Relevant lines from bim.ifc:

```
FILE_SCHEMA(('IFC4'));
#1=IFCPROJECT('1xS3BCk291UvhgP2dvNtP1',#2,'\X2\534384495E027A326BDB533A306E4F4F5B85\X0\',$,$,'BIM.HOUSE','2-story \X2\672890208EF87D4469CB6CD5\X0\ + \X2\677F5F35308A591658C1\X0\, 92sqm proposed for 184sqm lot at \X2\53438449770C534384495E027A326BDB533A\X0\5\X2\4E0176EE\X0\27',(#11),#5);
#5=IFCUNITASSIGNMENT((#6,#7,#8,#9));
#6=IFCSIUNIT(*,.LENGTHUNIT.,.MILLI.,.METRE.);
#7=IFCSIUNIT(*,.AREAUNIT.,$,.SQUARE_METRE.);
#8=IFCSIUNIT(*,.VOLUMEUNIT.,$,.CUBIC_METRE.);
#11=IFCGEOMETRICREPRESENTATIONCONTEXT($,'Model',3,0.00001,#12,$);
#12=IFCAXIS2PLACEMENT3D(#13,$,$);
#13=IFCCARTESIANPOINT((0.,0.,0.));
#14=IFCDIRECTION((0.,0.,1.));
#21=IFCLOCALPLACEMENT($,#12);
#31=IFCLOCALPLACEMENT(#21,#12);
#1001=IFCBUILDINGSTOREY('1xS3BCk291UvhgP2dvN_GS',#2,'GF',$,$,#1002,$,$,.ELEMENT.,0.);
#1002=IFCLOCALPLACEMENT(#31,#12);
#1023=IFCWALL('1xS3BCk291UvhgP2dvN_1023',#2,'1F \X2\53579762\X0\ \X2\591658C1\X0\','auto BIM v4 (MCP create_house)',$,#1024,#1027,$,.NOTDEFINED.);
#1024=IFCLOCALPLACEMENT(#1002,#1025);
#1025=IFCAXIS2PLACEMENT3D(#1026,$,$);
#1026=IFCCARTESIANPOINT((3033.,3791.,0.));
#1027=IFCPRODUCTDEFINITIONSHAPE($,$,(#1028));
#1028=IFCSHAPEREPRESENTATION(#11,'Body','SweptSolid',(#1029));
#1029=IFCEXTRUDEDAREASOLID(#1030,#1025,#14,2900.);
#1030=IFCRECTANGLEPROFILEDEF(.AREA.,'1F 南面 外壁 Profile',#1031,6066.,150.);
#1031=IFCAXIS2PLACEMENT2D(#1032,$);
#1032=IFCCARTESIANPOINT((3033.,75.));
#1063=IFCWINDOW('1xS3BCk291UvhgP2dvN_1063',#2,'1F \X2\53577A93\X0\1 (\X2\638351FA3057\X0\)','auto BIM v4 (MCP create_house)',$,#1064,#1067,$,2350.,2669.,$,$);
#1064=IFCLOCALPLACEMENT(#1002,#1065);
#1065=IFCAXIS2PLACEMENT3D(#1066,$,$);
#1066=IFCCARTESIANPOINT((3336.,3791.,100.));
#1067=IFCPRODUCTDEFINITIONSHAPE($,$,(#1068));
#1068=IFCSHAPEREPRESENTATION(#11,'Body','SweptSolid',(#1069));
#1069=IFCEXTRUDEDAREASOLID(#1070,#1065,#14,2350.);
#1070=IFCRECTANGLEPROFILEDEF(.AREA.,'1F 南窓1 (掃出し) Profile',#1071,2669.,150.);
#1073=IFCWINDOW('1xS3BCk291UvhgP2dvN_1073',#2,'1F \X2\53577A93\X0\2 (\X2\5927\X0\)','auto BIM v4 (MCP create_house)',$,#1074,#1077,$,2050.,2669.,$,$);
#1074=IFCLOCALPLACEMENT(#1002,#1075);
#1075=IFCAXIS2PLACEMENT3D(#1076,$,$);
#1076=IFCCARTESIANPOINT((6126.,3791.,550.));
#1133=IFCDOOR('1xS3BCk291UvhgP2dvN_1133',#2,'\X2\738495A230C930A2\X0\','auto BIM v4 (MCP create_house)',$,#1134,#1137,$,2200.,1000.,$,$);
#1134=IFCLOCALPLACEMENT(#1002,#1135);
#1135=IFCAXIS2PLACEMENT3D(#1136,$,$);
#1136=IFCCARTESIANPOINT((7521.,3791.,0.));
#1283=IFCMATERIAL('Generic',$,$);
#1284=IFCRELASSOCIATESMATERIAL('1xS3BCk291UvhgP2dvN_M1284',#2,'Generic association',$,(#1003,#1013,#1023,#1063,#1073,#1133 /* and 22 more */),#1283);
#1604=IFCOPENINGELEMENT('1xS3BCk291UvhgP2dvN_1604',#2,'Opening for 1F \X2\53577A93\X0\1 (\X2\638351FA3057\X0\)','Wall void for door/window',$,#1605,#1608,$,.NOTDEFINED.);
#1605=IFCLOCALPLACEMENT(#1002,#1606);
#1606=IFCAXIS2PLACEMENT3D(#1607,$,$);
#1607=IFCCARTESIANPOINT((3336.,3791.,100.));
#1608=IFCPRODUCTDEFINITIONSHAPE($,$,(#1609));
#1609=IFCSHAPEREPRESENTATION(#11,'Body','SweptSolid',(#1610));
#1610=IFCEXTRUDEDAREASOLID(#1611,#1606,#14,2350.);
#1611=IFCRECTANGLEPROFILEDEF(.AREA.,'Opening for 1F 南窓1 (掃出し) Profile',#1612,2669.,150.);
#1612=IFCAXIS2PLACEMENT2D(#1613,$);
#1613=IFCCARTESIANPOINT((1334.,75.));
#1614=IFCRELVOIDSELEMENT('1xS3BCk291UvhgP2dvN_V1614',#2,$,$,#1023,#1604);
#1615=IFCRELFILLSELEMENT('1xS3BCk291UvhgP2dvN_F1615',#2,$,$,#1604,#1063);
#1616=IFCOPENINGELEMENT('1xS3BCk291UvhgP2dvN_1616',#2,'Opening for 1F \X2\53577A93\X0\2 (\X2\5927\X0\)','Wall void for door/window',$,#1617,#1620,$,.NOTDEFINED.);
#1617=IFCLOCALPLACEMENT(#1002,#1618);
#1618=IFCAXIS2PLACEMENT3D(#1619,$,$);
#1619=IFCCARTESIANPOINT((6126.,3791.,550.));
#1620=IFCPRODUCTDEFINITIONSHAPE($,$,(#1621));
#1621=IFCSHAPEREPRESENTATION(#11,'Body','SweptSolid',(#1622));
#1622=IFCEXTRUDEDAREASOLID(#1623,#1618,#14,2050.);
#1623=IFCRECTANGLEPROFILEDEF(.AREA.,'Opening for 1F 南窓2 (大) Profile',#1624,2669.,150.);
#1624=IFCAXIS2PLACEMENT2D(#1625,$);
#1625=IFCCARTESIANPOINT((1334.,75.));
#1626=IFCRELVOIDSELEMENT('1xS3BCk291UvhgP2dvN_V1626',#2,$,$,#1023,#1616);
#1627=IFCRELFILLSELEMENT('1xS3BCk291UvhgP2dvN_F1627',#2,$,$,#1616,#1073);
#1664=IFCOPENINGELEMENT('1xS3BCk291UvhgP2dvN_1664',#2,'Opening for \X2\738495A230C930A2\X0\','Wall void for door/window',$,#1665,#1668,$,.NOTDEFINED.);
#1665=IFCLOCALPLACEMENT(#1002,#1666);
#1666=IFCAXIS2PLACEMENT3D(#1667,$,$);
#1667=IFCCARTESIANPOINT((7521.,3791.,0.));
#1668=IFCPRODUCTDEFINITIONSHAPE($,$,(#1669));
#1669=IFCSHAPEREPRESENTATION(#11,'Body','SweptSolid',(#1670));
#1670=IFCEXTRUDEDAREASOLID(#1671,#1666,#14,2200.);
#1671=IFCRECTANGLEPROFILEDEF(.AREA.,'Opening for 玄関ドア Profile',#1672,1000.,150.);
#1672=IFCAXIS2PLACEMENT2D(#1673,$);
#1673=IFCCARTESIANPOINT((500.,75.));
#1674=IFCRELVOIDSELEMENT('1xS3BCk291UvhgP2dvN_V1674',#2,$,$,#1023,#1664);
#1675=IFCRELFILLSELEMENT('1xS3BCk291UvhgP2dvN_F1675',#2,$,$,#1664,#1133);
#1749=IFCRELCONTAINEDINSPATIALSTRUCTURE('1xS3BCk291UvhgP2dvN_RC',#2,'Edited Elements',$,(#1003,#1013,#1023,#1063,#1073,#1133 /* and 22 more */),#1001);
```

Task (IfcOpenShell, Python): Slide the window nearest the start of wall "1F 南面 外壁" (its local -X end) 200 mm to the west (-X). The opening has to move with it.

```python
import ifcopenshell
import ifcopenshell.api.geometry
import ifcopenshell.util.placement

model = ifcopenshell.open("bim.ifc")

window = model.by_id(1063)
opening = window.FillsVoids[0].RelatingOpeningElement
wall = opening.VoidsElements[0].RelatingBuildingElement

wall_matrix = ifcopenshell.util.placement.get_local_placement(wall.ObjectPlacement)
shift = wall_matrix[:3, 0] * -200.0
before = ifcopenshell.util.placement.get_local_placement(window.ObjectPlacement)[:3, 3].copy()

# The window is not placed relative to its opening, so move both.
for product in (opening, window):
    matrix = ifcopenshell.util.placement.get_local_placement(product.ObjectPlacement)
    matrix[:3, 3] += shift
    ifcopenshell.api.geometry.edit_object_placement(model, product=product, matrix=matrix, is_si=False)

after = ifcopenshell.util.placement.get_local_placement(window.ObjectPlacement)[:3, 3]
print("window moved by", (after - before).round(3) + 0.0)

model.write("bim_edited.ifc")
```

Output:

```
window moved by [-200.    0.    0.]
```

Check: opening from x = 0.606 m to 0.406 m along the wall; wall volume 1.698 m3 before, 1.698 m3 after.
